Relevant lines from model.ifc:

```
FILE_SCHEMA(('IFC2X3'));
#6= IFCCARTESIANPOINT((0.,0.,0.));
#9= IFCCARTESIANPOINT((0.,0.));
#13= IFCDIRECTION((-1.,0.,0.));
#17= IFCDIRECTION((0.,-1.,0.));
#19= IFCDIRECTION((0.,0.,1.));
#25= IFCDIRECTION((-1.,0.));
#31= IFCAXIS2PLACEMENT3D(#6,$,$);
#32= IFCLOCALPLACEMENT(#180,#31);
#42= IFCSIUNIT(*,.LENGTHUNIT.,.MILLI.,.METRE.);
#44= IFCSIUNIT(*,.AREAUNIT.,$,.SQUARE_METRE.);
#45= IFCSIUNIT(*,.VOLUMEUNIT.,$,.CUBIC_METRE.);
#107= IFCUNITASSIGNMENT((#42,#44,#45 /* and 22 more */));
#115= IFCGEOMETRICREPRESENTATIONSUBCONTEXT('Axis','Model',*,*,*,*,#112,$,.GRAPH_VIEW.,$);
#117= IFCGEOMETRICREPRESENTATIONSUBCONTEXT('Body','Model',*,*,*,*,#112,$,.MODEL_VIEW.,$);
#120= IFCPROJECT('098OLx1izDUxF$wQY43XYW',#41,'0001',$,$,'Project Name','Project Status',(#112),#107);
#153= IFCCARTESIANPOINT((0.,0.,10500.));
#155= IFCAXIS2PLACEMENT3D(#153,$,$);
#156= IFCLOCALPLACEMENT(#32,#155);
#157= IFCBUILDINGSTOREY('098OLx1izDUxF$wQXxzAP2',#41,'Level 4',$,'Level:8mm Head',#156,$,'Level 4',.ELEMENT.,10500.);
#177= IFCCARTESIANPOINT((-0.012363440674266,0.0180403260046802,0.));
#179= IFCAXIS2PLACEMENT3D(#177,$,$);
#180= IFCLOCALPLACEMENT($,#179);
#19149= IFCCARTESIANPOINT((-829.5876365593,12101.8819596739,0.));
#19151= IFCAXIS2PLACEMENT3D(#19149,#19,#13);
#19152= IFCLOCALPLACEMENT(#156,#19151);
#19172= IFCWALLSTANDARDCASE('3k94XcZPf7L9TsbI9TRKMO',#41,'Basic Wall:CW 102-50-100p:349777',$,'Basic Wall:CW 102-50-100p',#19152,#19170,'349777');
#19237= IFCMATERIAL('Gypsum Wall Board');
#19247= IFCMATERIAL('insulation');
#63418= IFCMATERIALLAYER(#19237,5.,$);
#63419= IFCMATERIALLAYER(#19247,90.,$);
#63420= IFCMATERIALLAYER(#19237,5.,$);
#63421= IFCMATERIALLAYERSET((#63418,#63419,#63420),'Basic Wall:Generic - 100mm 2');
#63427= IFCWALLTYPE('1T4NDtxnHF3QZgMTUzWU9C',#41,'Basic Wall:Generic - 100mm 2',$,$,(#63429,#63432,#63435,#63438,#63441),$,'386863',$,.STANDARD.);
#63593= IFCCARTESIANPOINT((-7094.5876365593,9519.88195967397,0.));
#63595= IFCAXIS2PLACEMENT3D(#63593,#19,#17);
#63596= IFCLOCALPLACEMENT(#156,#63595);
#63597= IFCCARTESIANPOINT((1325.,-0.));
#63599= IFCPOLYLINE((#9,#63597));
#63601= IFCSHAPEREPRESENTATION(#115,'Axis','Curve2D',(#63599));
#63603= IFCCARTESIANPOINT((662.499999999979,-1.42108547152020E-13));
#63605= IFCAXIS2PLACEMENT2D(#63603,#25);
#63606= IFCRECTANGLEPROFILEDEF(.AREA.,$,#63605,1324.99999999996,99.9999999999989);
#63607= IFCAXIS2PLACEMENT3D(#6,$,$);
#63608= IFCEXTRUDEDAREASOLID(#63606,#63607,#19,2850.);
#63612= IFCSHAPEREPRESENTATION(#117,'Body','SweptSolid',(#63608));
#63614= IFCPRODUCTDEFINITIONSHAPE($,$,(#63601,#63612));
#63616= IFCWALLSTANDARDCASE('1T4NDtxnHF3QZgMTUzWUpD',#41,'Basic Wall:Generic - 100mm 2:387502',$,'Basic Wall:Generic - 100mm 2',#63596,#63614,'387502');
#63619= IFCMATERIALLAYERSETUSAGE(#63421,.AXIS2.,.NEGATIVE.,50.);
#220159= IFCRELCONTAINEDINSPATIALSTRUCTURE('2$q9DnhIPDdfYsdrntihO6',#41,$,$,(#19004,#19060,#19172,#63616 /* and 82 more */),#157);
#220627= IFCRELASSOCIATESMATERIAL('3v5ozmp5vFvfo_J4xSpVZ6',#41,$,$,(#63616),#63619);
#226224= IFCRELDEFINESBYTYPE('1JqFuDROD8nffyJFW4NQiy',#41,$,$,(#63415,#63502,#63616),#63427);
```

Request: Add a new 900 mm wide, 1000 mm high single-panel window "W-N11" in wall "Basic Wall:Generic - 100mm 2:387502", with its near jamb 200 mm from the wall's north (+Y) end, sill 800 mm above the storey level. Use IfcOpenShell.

```python
import numpy as np
import ifcopenshell
import ifcopenshell.api.feature
import ifcopenshell.api.geometry
import ifcopenshell.api.root
import ifcopenshell.api.spatial
import ifcopenshell.api.type
import ifcopenshell.geom
import ifcopenshell.util.element
import ifcopenshell.util.placement
import ifcopenshell.util.representation
import ifcopenshell.util.shape
import ifcopenshell.util.unit

model = ifcopenshell.open("model.ifc")
unit_scale = ifcopenshell.util.unit.calculate_unit_scale(model)
settings = ifcopenshell.geom.settings()


def volume(element):
    """Net volume in cubic metres, openings subtracted."""
    shape = ifcopenshell.geom.create_shape(settings, element)
    return ifcopenshell.util.shape.get_volume(shape.geometry)


wall = model.by_guid("1T4NDtxnHF3QZgMTUzWUpD")
storey = ifcopenshell.util.element.get_container(wall, ifc_class="IfcBuildingStorey")
context = ifcopenshell.util.representation.get_context(model, "Model", "Body", "MODEL_VIEW")
before = volume(wall)

width, height, from_end, sill = 0.9, 1, 0.2, 0.8  # metres

# The wall runs along its own X axis, and the end named is its -X end.
wall_shape = ifcopenshell.geom.create_shape(settings, wall)
x, y, z = ifcopenshell.util.shape.get_vertices(wall_shape.geometry).T
start = x.min() + from_end
face, thickness = float(y.min()), float(y.max() - y.min())
wall_matrix = ifcopenshell.util.placement.get_local_placement(wall.ObjectPlacement)
level = ifcopenshell.util.placement.get_local_placement(storey.ObjectPlacement)[2, 3]


def in_wall(x, y):
    """Placement at x, y metres in the wall's axes, at sill height."""
    matrix = wall_matrix.copy()
    matrix[:, 3] = wall_matrix @ np.array([x / unit_scale, y / unit_scale, 0.0, 1.0])
    matrix[2, 3] = level + sill / unit_scale
    return matrix


# Opening: a box that overshoots both wall faces by 50 mm.
opening = ifcopenshell.api.root.create_entity(model, ifc_class="IfcOpeningElement")
box = ifcopenshell.api.geometry.add_wall_representation(
    model, context=context, length=width, height=height, thickness=thickness + 0.1
)
ifcopenshell.api.geometry.assign_representation(model, product=opening, representation=box)
ifcopenshell.api.geometry.edit_object_placement(model, product=opening, matrix=in_wall(start, face - 0.05), is_si=False)
ifcopenshell.api.feature.add_feature(model, feature=opening, element=wall)

window = ifcopenshell.api.root.create_entity(model, ifc_class="IfcWindow", name="W-N11")
window.OverallWidth, window.OverallHeight = width / unit_scale, height / unit_scale
body = ifcopenshell.api.geometry.add_window_representation(
    model,
    context=context,
    overall_width=window.OverallWidth,
    overall_height=window.OverallHeight,
    partition_type="SINGLE_PANEL",
)
ifcopenshell.api.geometry.assign_representation(model, product=window, representation=body)
ifcopenshell.api.spatial.assign_container(model, products=[window], relating_structure=storey)
fills = ifcopenshell.api.feature.add_filling(model, opening=opening, element=window)
fills.OwnerHistory = window.OwnerHistory  # required in IFC2X3

# IFC2X3 keeps the operation on the window style.
style = ifcopenshell.api.root.create_entity(model, ifc_class="IfcWindowStyle", name="W-N11")
style.OperationType, style.ConstructionType = "SINGLE_PANEL", "NOTDEFINED"
style.ParameterTakesPrecedence = style.Sizeable = False
ifcopenshell.api.type.assign_type(model, related_objects=[window], relating_type=style)

# Centre the window in the wall's thickness.
ifcopenshell.api.geometry.edit_object_placement(model, product=window, matrix=in_wall(start, face), is_si=False)
window_shape = ifcopenshell.geom.create_shape(settings, window)
depth = ifcopenshell.util.shape.get_vertices(window_shape.geometry)[:, 1]
offset = face + thickness / 2 - (depth.min() + depth.max()) / 2
ifcopenshell.api.geometry.edit_object_placement(model, product=window, matrix=in_wall(start, offset), is_si=False)

after = volume(wall)

print(f"wall volume {before:.3f} -> {after:.3f} m3")

model.write("model_edited.ifc")
```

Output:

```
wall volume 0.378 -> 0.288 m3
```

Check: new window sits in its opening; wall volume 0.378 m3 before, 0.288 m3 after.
